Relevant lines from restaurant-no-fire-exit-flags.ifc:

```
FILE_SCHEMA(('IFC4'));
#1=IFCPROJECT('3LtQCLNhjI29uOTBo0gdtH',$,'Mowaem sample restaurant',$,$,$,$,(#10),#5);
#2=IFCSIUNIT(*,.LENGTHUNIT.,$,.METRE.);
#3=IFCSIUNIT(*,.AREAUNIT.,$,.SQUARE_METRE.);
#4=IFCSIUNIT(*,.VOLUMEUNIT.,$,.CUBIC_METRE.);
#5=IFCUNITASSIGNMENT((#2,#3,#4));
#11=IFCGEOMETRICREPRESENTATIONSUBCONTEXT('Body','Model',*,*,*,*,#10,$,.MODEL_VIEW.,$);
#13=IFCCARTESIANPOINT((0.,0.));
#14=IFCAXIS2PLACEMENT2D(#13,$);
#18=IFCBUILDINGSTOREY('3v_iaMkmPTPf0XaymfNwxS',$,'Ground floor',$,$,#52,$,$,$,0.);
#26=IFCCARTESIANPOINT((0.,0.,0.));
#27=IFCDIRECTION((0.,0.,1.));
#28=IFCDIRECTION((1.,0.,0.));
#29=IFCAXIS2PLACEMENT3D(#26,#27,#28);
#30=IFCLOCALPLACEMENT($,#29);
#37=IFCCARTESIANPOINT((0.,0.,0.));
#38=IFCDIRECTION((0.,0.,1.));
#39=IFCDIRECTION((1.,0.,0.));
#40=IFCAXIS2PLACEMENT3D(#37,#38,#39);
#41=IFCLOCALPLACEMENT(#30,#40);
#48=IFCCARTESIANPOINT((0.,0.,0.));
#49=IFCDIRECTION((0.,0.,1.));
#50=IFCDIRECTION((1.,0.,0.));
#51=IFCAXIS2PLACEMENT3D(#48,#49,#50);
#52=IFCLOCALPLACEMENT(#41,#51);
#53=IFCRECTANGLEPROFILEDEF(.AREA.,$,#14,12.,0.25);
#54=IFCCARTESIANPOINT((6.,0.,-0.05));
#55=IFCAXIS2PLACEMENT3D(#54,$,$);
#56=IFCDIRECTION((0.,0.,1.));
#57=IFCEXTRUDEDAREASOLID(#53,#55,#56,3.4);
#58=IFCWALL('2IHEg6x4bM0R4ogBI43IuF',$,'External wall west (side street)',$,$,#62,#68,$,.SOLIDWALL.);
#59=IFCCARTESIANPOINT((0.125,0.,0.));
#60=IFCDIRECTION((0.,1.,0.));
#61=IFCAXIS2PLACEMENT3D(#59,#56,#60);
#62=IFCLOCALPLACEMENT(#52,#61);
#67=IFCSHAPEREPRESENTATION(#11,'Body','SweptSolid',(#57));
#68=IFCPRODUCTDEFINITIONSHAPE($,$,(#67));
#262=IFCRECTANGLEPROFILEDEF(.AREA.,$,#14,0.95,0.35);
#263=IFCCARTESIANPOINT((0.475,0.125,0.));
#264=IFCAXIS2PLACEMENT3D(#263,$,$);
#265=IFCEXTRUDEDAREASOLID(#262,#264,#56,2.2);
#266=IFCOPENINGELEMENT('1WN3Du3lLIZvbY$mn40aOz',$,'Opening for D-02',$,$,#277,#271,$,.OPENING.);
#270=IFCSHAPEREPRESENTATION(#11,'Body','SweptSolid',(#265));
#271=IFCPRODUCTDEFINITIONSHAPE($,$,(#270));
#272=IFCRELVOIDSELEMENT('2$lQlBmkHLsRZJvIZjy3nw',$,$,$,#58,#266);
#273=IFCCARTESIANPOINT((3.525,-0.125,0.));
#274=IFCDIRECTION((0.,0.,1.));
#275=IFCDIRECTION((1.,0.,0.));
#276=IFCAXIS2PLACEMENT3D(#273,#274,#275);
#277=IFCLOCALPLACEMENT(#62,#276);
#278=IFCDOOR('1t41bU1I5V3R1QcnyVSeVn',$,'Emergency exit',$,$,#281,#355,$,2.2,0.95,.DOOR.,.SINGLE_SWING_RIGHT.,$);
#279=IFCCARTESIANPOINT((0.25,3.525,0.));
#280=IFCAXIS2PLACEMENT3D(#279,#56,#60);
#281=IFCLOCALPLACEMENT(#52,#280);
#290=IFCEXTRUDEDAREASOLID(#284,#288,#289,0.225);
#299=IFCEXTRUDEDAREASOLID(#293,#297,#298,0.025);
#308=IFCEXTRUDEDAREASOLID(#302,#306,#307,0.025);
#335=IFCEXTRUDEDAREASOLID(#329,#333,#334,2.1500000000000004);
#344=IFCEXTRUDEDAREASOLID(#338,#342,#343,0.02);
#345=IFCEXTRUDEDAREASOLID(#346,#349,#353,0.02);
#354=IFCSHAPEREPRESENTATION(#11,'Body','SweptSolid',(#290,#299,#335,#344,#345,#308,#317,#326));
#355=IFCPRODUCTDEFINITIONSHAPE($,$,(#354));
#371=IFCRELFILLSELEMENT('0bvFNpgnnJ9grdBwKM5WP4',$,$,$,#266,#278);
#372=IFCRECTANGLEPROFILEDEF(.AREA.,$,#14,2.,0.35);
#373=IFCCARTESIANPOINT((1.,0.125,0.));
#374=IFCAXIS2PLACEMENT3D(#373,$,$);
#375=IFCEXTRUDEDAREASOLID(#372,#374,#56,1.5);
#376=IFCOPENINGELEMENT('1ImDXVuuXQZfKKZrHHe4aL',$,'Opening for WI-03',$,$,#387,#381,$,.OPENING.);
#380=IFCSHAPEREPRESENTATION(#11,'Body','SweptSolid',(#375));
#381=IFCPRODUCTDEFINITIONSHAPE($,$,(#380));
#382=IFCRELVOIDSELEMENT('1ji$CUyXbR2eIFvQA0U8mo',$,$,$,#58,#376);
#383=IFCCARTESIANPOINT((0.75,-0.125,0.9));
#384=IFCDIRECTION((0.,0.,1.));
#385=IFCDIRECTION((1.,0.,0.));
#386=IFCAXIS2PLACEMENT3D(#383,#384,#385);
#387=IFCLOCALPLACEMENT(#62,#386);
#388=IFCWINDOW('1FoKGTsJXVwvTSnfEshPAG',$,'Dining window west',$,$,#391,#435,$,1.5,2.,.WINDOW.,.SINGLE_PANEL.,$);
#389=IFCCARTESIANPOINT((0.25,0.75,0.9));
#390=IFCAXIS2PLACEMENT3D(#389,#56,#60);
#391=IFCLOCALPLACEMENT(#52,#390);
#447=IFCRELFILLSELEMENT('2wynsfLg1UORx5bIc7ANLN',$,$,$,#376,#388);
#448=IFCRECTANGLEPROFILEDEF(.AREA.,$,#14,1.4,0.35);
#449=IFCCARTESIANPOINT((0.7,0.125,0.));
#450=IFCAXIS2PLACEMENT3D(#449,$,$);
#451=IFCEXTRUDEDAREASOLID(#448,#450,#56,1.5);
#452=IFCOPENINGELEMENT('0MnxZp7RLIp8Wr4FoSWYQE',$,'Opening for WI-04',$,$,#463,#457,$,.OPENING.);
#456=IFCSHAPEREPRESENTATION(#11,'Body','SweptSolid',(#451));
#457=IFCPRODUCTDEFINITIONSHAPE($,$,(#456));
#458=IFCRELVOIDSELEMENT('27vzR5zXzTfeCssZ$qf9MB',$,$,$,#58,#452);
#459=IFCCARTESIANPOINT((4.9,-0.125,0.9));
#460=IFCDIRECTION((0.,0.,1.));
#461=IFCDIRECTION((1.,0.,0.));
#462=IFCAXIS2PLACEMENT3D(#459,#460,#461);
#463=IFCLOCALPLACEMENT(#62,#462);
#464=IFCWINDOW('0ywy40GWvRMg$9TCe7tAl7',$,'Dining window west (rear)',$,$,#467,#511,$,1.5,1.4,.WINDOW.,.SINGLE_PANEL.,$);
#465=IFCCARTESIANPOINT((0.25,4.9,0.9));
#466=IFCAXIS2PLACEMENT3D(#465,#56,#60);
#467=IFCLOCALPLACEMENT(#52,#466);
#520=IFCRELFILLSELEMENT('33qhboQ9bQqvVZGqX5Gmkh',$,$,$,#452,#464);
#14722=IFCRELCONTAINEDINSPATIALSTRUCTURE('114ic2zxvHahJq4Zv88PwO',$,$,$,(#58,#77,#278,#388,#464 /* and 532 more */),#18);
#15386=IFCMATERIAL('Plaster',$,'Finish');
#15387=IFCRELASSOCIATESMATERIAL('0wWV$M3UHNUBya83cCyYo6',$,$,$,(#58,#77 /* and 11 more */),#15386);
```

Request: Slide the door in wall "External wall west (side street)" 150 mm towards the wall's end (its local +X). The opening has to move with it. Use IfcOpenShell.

```python
import ifcopenshell
import ifcopenshell.api.geometry
import ifcopenshell.util.placement
import ifcopenshell.util.unit

model = ifcopenshell.open("restaurant-no-fire-exit-flags.ifc")
unit_scale = ifcopenshell.util.unit.calculate_unit_scale(model)

door = model.by_guid("1t41bU1I5V3R1QcnyVSeVn")
opening = door.FillsVoids[0].RelatingOpeningElement
wall = opening.VoidsElements[0].RelatingBuildingElement

wall_matrix = ifcopenshell.util.placement.get_local_placement(wall.ObjectPlacement)
shift = wall_matrix[:3, 0] * 0.15 / unit_scale
before = ifcopenshell.util.placement.get_local_placement(door.ObjectPlacement)[:3, 3].copy()

# The door is not placed relative to its opening, so move both.
for product in (opening, door):
    matrix = ifcopenshell.util.placement.get_local_placement(product.ObjectPlacement)
    matrix[:3, 3] += shift
    ifcopenshell.api.geometry.edit_object_placement(model, product=product, matrix=matrix, is_si=False)

after = ifcopenshell.util.placement.get_local_placement(door.ObjectPlacement)[:3, 3]
print("door moved by", (after - before).round(3) + 0.0)

model.write("restaurant-no-fire-exit-flags_edited.ifc")
```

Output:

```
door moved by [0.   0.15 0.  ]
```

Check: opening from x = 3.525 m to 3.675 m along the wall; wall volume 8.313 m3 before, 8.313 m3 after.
